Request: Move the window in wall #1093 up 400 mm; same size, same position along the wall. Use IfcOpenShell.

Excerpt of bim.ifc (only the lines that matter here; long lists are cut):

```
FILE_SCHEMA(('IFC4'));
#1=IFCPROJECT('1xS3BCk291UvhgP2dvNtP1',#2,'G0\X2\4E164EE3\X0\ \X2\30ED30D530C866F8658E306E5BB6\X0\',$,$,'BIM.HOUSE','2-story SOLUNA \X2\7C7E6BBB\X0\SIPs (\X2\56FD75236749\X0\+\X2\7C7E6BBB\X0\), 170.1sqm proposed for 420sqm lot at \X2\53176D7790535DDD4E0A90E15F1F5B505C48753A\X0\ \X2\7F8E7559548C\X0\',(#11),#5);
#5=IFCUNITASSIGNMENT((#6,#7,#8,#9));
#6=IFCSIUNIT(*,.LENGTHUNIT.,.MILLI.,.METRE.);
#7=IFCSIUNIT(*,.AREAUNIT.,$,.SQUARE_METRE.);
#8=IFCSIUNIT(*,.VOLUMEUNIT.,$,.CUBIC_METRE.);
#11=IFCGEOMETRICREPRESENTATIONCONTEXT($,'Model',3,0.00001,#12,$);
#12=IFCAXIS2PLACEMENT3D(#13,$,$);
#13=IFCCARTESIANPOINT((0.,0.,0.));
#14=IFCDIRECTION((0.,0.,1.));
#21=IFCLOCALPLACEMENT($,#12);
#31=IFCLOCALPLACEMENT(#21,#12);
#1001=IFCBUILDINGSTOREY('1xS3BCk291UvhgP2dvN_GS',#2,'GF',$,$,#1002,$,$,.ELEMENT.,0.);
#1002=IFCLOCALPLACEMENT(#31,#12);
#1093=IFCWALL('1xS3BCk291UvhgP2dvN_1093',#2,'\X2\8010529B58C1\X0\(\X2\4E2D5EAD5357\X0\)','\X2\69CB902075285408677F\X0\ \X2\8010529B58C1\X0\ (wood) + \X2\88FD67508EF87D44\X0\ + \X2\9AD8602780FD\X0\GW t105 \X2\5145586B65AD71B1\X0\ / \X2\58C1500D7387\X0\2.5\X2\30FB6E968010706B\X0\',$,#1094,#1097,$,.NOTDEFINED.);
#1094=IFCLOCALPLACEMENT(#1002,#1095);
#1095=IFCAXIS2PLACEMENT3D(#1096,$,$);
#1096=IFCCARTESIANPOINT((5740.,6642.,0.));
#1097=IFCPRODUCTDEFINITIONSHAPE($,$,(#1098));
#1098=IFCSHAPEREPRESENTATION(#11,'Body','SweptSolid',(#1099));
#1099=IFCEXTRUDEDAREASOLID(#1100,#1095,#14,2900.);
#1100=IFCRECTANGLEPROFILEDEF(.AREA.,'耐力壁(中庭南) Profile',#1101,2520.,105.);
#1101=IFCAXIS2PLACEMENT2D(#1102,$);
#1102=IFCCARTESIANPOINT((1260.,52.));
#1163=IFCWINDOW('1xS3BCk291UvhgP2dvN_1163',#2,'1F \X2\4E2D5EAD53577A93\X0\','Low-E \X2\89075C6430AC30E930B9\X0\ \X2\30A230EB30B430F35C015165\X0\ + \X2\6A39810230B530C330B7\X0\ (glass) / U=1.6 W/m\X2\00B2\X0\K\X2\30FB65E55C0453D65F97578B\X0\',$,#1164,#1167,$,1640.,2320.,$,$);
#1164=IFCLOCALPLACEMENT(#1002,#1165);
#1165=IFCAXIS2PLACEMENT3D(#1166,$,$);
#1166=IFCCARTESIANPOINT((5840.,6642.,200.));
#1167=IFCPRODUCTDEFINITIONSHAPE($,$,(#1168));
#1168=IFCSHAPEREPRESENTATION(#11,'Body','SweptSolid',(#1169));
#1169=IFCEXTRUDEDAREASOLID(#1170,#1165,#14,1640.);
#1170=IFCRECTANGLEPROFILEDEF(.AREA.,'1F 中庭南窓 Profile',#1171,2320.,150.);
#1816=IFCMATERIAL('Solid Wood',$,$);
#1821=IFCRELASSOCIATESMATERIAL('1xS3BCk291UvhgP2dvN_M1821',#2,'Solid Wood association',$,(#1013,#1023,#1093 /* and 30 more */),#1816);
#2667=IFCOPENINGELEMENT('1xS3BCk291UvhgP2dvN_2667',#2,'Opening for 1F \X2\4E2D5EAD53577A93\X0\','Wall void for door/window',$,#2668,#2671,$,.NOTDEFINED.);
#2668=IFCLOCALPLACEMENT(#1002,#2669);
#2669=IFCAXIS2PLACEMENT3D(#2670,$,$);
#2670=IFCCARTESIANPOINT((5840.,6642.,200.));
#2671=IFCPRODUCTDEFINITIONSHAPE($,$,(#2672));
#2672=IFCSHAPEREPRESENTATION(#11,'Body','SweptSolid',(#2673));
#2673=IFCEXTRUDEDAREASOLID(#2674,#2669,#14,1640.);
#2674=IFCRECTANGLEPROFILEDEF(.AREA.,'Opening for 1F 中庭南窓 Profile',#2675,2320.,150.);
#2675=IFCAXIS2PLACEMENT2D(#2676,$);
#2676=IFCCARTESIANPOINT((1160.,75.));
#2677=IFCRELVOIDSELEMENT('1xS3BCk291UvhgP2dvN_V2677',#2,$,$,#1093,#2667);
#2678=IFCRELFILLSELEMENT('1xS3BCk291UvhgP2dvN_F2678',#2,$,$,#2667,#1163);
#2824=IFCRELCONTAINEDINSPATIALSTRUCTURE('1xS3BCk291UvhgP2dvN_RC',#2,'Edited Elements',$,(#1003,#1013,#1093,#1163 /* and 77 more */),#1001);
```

```python
import numpy as np
import ifcopenshell
import ifcopenshell.api.geometry
import ifcopenshell.util.placement
import ifcopenshell.util.unit

model = ifcopenshell.open("bim.ifc")
unit_scale = ifcopenshell.util.unit.calculate_unit_scale(model)

window = model.by_guid("1xS3BCk291UvhgP2dvN_1163")
opening = window.FillsVoids[0].RelatingOpeningElement
dz = 400.0

shift = np.array([0.0, 0.0, dz])
# The window is not placed relative to its opening, so move both.
for product in (opening, window):
    matrix = ifcopenshell.util.placement.get_local_placement(product.ObjectPlacement)
    matrix[:3, 3] += shift
    ifcopenshell.api.geometry.edit_object_placement(model, product=product, matrix=matrix, is_si=False)

print(f"moved by {dz * unit_scale:+.3f} m")

model.write("bim_rev.ifc")
```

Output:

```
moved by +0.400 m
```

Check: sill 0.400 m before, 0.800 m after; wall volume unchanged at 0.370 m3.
